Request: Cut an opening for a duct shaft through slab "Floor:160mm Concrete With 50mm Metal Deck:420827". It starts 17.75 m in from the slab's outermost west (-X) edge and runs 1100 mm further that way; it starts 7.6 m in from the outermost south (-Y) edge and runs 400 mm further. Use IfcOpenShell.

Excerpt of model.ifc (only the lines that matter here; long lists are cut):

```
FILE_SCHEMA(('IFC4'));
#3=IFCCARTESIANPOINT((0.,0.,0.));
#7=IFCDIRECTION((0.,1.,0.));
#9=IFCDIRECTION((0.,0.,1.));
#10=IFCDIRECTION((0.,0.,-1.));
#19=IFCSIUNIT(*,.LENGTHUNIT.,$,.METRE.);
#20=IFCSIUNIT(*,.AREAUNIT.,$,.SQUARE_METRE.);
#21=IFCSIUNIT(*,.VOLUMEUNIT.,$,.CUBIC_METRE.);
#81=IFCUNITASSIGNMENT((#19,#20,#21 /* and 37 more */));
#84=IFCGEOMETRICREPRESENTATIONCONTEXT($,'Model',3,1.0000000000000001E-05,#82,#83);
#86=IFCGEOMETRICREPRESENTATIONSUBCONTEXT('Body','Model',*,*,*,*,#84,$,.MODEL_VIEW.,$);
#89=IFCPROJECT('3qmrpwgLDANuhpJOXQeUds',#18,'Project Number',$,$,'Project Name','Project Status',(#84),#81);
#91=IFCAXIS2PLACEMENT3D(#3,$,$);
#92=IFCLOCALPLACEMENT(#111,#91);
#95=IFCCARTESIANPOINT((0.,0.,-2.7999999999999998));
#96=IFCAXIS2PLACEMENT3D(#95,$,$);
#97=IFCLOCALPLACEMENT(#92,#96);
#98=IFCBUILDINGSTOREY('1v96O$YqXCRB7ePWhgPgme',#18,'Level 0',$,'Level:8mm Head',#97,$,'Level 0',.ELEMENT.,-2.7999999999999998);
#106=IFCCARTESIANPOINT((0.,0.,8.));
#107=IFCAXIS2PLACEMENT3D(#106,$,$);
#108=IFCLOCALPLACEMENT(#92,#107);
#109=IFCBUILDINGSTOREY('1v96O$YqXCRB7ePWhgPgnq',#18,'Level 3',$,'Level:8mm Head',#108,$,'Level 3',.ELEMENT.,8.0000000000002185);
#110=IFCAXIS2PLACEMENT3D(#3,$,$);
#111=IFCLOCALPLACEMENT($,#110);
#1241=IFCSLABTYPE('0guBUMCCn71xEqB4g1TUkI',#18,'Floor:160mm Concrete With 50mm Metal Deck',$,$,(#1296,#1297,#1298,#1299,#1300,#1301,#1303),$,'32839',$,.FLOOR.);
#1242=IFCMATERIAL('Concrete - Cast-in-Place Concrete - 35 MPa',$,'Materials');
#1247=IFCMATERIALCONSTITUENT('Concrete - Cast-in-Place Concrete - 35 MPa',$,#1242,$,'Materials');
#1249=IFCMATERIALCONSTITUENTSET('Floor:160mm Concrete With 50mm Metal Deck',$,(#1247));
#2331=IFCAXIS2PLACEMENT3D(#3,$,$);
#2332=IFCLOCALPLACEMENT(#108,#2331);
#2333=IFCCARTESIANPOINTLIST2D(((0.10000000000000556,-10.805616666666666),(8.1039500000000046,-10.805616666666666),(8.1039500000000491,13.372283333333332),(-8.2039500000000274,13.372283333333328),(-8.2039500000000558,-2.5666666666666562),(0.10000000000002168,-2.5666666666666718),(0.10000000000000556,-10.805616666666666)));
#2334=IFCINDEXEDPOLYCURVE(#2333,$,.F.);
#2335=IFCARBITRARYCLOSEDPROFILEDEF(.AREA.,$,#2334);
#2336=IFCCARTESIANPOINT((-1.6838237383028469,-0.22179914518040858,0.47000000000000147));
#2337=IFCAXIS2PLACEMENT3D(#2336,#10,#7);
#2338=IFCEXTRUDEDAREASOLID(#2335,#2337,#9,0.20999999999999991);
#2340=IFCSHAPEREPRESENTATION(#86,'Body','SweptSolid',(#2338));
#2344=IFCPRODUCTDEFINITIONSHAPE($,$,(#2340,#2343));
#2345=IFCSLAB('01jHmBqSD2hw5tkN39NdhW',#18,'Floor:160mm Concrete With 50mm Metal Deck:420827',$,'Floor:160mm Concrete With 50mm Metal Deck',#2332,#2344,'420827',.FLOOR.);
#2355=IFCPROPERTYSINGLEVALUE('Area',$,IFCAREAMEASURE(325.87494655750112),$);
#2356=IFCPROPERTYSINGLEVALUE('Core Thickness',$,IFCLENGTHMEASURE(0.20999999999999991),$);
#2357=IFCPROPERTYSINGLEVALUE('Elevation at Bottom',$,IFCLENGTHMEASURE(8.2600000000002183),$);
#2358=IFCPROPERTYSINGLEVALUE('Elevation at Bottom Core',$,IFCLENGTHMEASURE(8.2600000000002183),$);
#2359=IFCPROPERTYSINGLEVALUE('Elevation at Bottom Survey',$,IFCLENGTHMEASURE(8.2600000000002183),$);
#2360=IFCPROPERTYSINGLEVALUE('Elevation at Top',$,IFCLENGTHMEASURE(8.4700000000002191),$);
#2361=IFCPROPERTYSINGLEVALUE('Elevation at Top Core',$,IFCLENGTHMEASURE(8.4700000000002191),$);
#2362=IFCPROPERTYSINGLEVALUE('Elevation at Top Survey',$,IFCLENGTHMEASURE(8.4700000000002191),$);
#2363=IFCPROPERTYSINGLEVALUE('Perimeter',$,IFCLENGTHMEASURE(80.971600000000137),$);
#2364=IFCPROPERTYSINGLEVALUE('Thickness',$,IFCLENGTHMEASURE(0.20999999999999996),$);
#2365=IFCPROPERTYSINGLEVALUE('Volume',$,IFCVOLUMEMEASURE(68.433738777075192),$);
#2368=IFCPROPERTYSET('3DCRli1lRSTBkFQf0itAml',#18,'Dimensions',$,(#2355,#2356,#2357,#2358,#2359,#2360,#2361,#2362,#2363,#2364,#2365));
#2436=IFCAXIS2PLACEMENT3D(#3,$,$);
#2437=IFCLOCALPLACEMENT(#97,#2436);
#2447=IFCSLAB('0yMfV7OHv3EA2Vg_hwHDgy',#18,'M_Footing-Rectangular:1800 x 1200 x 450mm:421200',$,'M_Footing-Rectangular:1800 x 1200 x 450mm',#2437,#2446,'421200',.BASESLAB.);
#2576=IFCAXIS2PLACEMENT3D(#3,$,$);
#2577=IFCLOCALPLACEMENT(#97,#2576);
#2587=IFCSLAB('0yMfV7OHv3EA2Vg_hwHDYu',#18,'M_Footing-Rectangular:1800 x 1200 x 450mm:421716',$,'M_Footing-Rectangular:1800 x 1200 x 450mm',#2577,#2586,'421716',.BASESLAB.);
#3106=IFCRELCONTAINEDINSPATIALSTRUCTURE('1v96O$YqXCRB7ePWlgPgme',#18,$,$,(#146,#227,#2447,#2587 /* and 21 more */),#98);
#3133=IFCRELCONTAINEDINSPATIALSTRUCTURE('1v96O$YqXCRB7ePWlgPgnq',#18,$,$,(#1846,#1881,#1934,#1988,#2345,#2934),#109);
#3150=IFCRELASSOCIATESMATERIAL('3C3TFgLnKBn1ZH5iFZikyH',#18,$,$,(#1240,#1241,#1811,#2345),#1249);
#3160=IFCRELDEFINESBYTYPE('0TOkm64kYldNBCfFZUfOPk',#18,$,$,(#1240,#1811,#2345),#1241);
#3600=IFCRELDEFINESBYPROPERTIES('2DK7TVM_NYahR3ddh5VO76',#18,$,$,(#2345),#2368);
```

```python
import numpy as np
import ifcopenshell
import ifcopenshell.api.feature
import ifcopenshell.api.geometry
import ifcopenshell.api.pset
import ifcopenshell.api.root
import ifcopenshell.geom
import ifcopenshell.util.element
import ifcopenshell.util.placement
import ifcopenshell.util.representation
import ifcopenshell.util.shape
import ifcopenshell.util.unit

model = ifcopenshell.open("model.ifc")
unit_scale = ifcopenshell.util.unit.calculate_unit_scale(model)
area_scale = ifcopenshell.util.unit.calculate_unit_scale(model, "AREAUNIT")
volume_scale = ifcopenshell.util.unit.calculate_unit_scale(model, "VOLUMEUNIT")
settings = ifcopenshell.geom.settings()


def volume(element):
    """Net volume in cubic metres, openings subtracted."""
    shape = ifcopenshell.geom.create_shape(settings, element)
    return ifcopenshell.util.shape.get_volume(shape.geometry)


slab = model.by_id(2345)
before = volume(slab)

# Extent in the slab's own axes, in metres. The edges named are its -X and -Y sides.
slab_shape = ifcopenshell.geom.create_shape(settings, slab)
vertices = ifcopenshell.util.shape.get_vertices(slab_shape.geometry)
x_min, y_min, bottom = vertices.min(axis=0)
top = vertices[:, 2].max()

opening = ifcopenshell.api.root.create_entity(model, ifc_class="IfcOpeningElement", name="Duct shaft opening", predefined_type="OPENING")
context = ifcopenshell.util.representation.get_context(model, "Model", "Body", "MODEL_VIEW")
width, depth = 1.1, 0.4
outline = [(0.0, 0.0), (width, 0.0), (width, depth), (0.0, depth), (0.0, 0.0)]
# Overshoot both faces by 50 mm so the cut is clean.
shape = ifcopenshell.api.geometry.add_slab_representation(
    model, context=context, depth=top - bottom + 0.1, polyline=outline
)
ifcopenshell.api.geometry.assign_representation(model, product=opening, representation=shape)

matrix = ifcopenshell.util.placement.get_local_placement(slab.ObjectPlacement)
matrix[:, 3] = matrix @ np.append(np.array([x_min + 17.75, y_min + 7.6, bottom - 0.05]) / unit_scale, 1.0)
ifcopenshell.api.geometry.edit_object_placement(model, product=opening, matrix=matrix, is_si=False)
ifcopenshell.api.feature.add_feature(model, feature=opening, element=slab)

after = volume(slab)

# Update the slab's stored quantities.
pset = model.by_id(ifcopenshell.util.element.get_pset(slab, "Dimensions", should_inherit=False)["id"])
ifcopenshell.api.pset.edit_pset(model, pset=pset, properties={
    "Area": model.create_entity("IfcAreaMeasure", after / (top - bottom) / area_scale),
    "Volume": model.create_entity("IfcVolumeMeasure", after / volume_scale),
})

print(f"slab volume {before:.3f} -> {after:.3f} m3")

model.write("model-out.ifc")
```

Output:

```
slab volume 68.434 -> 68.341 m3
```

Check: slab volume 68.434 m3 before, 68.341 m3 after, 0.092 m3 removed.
